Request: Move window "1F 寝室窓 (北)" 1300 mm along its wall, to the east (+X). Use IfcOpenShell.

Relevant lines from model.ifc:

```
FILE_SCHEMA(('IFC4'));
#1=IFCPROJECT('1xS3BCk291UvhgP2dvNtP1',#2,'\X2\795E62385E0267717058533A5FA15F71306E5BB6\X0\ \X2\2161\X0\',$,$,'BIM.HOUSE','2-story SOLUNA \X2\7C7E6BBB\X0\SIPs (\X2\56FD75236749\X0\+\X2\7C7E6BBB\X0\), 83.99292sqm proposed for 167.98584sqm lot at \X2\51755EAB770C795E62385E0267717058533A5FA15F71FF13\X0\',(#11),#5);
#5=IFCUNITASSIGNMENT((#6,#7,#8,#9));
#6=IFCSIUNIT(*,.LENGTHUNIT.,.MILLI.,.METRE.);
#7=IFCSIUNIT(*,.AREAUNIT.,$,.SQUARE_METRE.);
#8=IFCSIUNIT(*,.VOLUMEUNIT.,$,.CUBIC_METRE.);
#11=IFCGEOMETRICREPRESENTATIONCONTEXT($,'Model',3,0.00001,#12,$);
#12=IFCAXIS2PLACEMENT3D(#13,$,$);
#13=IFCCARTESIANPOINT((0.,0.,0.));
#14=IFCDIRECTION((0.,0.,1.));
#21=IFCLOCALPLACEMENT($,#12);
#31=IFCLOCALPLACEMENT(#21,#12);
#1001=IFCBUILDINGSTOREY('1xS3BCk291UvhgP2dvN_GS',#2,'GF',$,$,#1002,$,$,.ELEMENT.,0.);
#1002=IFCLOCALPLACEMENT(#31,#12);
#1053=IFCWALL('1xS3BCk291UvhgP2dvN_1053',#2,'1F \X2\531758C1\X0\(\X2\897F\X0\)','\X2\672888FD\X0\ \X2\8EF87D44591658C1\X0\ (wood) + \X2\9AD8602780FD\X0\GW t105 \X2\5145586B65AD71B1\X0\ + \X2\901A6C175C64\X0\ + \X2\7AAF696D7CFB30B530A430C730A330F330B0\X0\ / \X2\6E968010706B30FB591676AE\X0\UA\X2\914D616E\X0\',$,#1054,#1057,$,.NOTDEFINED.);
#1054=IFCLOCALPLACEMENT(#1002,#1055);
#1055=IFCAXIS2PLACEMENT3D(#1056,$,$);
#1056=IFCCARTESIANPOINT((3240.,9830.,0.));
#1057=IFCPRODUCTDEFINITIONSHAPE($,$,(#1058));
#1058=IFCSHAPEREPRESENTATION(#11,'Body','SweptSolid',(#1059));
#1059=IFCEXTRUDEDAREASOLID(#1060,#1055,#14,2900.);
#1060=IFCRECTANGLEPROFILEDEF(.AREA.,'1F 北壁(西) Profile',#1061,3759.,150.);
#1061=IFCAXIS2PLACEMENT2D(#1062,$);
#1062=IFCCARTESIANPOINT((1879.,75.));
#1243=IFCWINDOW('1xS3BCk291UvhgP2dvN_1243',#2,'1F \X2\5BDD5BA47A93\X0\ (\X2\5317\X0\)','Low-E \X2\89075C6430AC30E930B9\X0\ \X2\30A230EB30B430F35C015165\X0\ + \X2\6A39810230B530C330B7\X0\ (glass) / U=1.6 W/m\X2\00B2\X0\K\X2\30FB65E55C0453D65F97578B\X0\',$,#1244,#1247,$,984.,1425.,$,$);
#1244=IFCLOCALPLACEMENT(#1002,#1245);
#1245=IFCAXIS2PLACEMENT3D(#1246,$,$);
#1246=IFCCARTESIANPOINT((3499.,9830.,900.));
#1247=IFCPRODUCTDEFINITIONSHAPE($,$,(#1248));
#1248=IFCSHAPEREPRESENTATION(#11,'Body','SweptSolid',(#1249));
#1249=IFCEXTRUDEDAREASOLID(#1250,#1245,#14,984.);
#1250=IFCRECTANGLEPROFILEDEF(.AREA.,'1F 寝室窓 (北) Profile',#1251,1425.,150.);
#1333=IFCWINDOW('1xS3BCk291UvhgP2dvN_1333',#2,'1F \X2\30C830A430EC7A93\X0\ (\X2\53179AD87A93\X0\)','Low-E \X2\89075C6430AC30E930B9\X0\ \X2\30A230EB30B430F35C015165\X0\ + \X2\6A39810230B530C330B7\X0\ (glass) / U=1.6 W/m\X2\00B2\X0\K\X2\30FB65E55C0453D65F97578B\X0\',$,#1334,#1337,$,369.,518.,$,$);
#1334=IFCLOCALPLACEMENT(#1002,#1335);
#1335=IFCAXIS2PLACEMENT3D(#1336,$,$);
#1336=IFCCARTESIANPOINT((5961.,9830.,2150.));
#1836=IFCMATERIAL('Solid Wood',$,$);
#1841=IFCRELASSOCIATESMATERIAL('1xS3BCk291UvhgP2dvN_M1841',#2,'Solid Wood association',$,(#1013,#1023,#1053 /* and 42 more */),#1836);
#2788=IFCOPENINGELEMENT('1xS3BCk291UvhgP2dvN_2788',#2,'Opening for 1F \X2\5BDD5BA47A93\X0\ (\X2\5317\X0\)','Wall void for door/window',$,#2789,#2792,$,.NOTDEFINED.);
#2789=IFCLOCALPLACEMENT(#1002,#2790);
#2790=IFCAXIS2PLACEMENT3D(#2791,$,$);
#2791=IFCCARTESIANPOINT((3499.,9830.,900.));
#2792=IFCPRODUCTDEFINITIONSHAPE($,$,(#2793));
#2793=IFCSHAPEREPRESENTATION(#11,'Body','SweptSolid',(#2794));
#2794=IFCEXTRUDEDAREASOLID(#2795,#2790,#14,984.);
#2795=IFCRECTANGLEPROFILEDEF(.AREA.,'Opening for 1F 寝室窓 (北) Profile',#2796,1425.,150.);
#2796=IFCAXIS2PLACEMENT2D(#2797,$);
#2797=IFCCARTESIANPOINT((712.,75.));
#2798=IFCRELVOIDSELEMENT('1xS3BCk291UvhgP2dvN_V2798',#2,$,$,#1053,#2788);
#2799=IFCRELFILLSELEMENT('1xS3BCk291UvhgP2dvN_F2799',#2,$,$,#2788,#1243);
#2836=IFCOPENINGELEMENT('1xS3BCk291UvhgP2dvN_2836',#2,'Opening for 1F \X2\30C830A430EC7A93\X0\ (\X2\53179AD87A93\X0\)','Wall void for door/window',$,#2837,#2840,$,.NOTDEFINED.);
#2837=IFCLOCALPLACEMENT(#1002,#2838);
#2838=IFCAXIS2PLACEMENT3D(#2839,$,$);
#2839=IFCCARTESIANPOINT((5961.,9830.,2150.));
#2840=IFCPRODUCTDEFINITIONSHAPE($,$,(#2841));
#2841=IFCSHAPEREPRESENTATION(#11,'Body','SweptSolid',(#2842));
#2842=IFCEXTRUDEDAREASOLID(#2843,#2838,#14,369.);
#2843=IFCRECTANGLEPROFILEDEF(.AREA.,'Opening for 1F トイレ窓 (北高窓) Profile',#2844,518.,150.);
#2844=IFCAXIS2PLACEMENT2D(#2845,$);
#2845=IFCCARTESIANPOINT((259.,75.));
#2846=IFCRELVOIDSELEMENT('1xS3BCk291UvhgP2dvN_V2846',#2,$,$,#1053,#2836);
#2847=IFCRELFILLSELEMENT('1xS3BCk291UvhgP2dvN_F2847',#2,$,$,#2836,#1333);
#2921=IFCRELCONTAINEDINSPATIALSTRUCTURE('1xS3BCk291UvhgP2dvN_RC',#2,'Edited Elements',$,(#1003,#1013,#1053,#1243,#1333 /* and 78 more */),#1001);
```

```python
import ifcopenshell
import ifcopenshell.api.geometry
import ifcopenshell.util.placement
import ifcopenshell.util.unit

model = ifcopenshell.open("model.ifc")
unit_scale = ifcopenshell.util.unit.calculate_unit_scale(model)

window = model.by_guid("1xS3BCk291UvhgP2dvN_1243")
opening = window.FillsVoids[0].RelatingOpeningElement
wall = opening.VoidsElements[0].RelatingBuildingElement

wall_matrix = ifcopenshell.util.placement.get_local_placement(wall.ObjectPlacement)
shift = wall_matrix[:3, 0] * 1.3 / unit_scale
before = ifcopenshell.util.placement.get_local_placement(window.ObjectPlacement)[:3, 3].copy()

# The window is not placed relative to its opening, so move both.
for product in (opening, window):
    matrix = ifcopenshell.util.placement.get_local_placement(product.ObjectPlacement)
    matrix[:3, 3] += shift
    ifcopenshell.api.geometry.edit_object_placement(model, product=product, matrix=matrix, is_si=False)

after = ifcopenshell.util.placement.get_local_placement(window.ObjectPlacement)[:3, 3]
print("window moved by", (after - before).round(3) + 0.0)

model.write("model_rev.ifc")
```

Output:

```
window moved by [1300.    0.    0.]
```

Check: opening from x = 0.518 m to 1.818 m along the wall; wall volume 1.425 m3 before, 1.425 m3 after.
